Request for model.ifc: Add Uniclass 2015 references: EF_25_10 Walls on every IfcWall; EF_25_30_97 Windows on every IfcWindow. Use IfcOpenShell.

First a look at what the model holds.

```python
import ifcopenshell

model = ifcopenshell.open("model.ifc")
print(model.schema)
print("classifications:", [c.Name for c in model.by_type("IfcClassification")])
for ifc_class in ("IfcDoor", "IfcRoof", "IfcStair", "IfcWall", "IfcWindow"):
    print(ifc_class, len(model.by_type(ifc_class)))
```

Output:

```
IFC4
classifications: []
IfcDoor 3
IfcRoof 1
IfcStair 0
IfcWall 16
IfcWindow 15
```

```python
import ifcopenshell
import ifcopenshell.api.classification

model = ifcopenshell.open("model.ifc")

system = ifcopenshell.api.classification.add_classification(model, classification="Uniclass 2015")

codes = {
    "IfcWall": ("EF_25_10", "Walls"),
    "IfcWindow": ("EF_25_30_97", "Windows"),
}
for ifc_class, (code, name) in codes.items():
    products = model.by_type(ifc_class)
    ifcopenshell.api.classification.add_reference(
        model, products=products, classification=system, identification=code, name=name
    )
    print(code, len(products))

model.write("model_rev.ifc")
```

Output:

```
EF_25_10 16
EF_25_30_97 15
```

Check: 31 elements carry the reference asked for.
